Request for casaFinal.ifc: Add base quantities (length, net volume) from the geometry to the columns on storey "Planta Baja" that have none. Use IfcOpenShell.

First a look at what the model holds.

```python
import ifcopenshell
import ifcopenshell.util.element
import ifcopenshell.util.unit

model = ifcopenshell.open("casaFinal.ifc")
print(model.schema)
for unit_type in ("LENGTHUNIT", "AREAUNIT", "VOLUMEUNIT"):
    print(unit_type, ifcopenshell.util.unit.calculate_unit_scale(model, unit_type))
storey = next(s for s in model.by_type("IfcBuildingStorey") if s.Name == "Planta Baja")
columns = [e for e in ifcopenshell.util.element.get_decomposition(storey) if e.is_a("IfcColumn")]
for e in sorted(columns, key=lambda e: e.id()):
    print(e.id(), e.is_a(), e.Name, list(ifcopenshell.util.element.get_psets(e, qtos_only=True)), sep=" | ")
```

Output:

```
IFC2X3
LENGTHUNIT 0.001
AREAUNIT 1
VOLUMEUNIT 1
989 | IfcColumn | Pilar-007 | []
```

```python
import ifcopenshell
import ifcopenshell.api.pset
import ifcopenshell.geom
import ifcopenshell.util.element
import ifcopenshell.util.shape
import ifcopenshell.util.unit

model = ifcopenshell.open("casaFinal.ifc")
unit_scale = ifcopenshell.util.unit.calculate_unit_scale(model)
volume_scale = ifcopenshell.util.unit.calculate_unit_scale(model, "VOLUMEUNIT")
settings = ifcopenshell.geom.settings()

storey = next(s for s in model.by_type("IfcBuildingStorey") if s.Name == "Planta Baja")
columns = [e for e in ifcopenshell.util.element.get_decomposition(storey) if e.is_a("IfcColumn")]

for e in sorted(columns, key=lambda e: e.id()):
    if ifcopenshell.util.element.get_psets(e, qtos_only=True, should_inherit=False):
        continue
    # Geometry comes back in metres, in the element's own axes.
    shape = ifcopenshell.geom.create_shape(settings, e)
    values = {
        "Length": ifcopenshell.util.shape.get_z(shape.geometry) / unit_scale,
        "NetVolume": ifcopenshell.util.shape.get_volume(shape.geometry) / volume_scale,
    }
    qto = ifcopenshell.api.pset.add_qto(model, product=e, name="BaseQuantities")
    ifcopenshell.api.pset.edit_qto(model, qto=qto, properties=values)
    print(e.id(), {k: round(v, 3) for k, v in values.items()})

model.write("casaFinal_edited.ifc")
```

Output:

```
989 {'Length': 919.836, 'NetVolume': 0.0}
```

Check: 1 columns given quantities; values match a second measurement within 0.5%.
